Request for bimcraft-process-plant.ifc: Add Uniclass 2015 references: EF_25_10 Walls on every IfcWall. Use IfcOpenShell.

First a look at what the model holds.

```python
import ifcopenshell

model = ifcopenshell.open("bimcraft-process-plant.ifc")
print(model.schema)
print("classifications:", [c.Name for c in model.by_type("IfcClassification")])
for ifc_class in ("IfcDoor", "IfcRoof", "IfcStair", "IfcWall", "IfcWindow"):
    print(ifc_class, len(model.by_type(ifc_class)))
```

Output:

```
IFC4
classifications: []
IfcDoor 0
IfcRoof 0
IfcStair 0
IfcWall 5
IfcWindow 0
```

```python
import ifcopenshell
import ifcopenshell.api.classification

model = ifcopenshell.open("bimcraft-process-plant.ifc")

system = ifcopenshell.api.classification.add_classification(model, classification="Uniclass 2015")

codes = {
    "IfcWall": ("EF_25_10", "Walls"),
}
for ifc_class, (code, name) in codes.items():
    products = model.by_type(ifc_class)
    ifcopenshell.api.classification.add_reference(
        model, products=products, classification=system, identification=code, name=name
    )
    print(code, len(products))

model.write("bimcraft-process-plant_edited.ifc")
```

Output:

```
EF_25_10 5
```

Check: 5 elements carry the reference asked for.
